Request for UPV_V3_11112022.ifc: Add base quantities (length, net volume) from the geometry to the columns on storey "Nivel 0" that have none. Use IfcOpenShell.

First a look at what the model holds.

```python
import ifcopenshell
import ifcopenshell.util.element
import ifcopenshell.util.unit

model = ifcopenshell.open("UPV_V3_11112022.ifc")
print(model.schema)
for unit_type in ("LENGTHUNIT", "AREAUNIT", "VOLUMEUNIT"):
    print(unit_type, ifcopenshell.util.unit.calculate_unit_scale(model, unit_type))
storey = next(s for s in model.by_type("IfcBuildingStorey") if s.Name == "Nivel 0")
columns = [e for e in ifcopenshell.util.element.get_decomposition(storey) if e.is_a("IfcColumn")]
for e in sorted(columns, key=lambda e: e.id()):
    print(e.id(), e.is_a(), e.Name, list(ifcopenshell.util.element.get_psets(e, qtos_only=True)), sep=" | ")
```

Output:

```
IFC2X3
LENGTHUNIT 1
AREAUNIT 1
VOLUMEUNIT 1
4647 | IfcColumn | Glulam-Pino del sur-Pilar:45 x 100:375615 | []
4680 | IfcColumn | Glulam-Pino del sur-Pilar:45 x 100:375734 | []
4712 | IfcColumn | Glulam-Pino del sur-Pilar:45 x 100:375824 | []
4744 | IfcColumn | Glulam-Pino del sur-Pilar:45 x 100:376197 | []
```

```python
import ifcopenshell
import ifcopenshell.api.pset
import ifcopenshell.geom
import ifcopenshell.util.element
import ifcopenshell.util.shape
import ifcopenshell.util.unit

model = ifcopenshell.open("UPV_V3_11112022.ifc")
unit_scale = ifcopenshell.util.unit.calculate_unit_scale(model)
volume_scale = ifcopenshell.util.unit.calculate_unit_scale(model, "VOLUMEUNIT")
settings = ifcopenshell.geom.settings()

storey = next(s for s in model.by_type("IfcBuildingStorey") if s.Name == "Nivel 0")
columns = [e for e in ifcopenshell.util.element.get_decomposition(storey) if e.is_a("IfcColumn")]

for e in sorted(columns, key=lambda e: e.id()):
    if ifcopenshell.util.element.get_psets(e, qtos_only=True, should_inherit=False):
        continue
    # Geometry comes back in metres, in the element's own axes.
    shape = ifcopenshell.geom.create_shape(settings, e)
    values = {
        "Length": ifcopenshell.util.shape.get_z(shape.geometry) / unit_scale,
        "NetVolume": ifcopenshell.util.shape.get_volume(shape.geometry) / volume_scale,
    }
    qto = ifcopenshell.api.pset.add_qto(model, product=e, name="BaseQuantities")
    ifcopenshell.api.pset.edit_qto(model, qto=qto, properties=values)
    print(e.id(), {k: round(v, 3) for k, v in values.items()})

model.write("UPV_V3_11112022_rev.ifc")
```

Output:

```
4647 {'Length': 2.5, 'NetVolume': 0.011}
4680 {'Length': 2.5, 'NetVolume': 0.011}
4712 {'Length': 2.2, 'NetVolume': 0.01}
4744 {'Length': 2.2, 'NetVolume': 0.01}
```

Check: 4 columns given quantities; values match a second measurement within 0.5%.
